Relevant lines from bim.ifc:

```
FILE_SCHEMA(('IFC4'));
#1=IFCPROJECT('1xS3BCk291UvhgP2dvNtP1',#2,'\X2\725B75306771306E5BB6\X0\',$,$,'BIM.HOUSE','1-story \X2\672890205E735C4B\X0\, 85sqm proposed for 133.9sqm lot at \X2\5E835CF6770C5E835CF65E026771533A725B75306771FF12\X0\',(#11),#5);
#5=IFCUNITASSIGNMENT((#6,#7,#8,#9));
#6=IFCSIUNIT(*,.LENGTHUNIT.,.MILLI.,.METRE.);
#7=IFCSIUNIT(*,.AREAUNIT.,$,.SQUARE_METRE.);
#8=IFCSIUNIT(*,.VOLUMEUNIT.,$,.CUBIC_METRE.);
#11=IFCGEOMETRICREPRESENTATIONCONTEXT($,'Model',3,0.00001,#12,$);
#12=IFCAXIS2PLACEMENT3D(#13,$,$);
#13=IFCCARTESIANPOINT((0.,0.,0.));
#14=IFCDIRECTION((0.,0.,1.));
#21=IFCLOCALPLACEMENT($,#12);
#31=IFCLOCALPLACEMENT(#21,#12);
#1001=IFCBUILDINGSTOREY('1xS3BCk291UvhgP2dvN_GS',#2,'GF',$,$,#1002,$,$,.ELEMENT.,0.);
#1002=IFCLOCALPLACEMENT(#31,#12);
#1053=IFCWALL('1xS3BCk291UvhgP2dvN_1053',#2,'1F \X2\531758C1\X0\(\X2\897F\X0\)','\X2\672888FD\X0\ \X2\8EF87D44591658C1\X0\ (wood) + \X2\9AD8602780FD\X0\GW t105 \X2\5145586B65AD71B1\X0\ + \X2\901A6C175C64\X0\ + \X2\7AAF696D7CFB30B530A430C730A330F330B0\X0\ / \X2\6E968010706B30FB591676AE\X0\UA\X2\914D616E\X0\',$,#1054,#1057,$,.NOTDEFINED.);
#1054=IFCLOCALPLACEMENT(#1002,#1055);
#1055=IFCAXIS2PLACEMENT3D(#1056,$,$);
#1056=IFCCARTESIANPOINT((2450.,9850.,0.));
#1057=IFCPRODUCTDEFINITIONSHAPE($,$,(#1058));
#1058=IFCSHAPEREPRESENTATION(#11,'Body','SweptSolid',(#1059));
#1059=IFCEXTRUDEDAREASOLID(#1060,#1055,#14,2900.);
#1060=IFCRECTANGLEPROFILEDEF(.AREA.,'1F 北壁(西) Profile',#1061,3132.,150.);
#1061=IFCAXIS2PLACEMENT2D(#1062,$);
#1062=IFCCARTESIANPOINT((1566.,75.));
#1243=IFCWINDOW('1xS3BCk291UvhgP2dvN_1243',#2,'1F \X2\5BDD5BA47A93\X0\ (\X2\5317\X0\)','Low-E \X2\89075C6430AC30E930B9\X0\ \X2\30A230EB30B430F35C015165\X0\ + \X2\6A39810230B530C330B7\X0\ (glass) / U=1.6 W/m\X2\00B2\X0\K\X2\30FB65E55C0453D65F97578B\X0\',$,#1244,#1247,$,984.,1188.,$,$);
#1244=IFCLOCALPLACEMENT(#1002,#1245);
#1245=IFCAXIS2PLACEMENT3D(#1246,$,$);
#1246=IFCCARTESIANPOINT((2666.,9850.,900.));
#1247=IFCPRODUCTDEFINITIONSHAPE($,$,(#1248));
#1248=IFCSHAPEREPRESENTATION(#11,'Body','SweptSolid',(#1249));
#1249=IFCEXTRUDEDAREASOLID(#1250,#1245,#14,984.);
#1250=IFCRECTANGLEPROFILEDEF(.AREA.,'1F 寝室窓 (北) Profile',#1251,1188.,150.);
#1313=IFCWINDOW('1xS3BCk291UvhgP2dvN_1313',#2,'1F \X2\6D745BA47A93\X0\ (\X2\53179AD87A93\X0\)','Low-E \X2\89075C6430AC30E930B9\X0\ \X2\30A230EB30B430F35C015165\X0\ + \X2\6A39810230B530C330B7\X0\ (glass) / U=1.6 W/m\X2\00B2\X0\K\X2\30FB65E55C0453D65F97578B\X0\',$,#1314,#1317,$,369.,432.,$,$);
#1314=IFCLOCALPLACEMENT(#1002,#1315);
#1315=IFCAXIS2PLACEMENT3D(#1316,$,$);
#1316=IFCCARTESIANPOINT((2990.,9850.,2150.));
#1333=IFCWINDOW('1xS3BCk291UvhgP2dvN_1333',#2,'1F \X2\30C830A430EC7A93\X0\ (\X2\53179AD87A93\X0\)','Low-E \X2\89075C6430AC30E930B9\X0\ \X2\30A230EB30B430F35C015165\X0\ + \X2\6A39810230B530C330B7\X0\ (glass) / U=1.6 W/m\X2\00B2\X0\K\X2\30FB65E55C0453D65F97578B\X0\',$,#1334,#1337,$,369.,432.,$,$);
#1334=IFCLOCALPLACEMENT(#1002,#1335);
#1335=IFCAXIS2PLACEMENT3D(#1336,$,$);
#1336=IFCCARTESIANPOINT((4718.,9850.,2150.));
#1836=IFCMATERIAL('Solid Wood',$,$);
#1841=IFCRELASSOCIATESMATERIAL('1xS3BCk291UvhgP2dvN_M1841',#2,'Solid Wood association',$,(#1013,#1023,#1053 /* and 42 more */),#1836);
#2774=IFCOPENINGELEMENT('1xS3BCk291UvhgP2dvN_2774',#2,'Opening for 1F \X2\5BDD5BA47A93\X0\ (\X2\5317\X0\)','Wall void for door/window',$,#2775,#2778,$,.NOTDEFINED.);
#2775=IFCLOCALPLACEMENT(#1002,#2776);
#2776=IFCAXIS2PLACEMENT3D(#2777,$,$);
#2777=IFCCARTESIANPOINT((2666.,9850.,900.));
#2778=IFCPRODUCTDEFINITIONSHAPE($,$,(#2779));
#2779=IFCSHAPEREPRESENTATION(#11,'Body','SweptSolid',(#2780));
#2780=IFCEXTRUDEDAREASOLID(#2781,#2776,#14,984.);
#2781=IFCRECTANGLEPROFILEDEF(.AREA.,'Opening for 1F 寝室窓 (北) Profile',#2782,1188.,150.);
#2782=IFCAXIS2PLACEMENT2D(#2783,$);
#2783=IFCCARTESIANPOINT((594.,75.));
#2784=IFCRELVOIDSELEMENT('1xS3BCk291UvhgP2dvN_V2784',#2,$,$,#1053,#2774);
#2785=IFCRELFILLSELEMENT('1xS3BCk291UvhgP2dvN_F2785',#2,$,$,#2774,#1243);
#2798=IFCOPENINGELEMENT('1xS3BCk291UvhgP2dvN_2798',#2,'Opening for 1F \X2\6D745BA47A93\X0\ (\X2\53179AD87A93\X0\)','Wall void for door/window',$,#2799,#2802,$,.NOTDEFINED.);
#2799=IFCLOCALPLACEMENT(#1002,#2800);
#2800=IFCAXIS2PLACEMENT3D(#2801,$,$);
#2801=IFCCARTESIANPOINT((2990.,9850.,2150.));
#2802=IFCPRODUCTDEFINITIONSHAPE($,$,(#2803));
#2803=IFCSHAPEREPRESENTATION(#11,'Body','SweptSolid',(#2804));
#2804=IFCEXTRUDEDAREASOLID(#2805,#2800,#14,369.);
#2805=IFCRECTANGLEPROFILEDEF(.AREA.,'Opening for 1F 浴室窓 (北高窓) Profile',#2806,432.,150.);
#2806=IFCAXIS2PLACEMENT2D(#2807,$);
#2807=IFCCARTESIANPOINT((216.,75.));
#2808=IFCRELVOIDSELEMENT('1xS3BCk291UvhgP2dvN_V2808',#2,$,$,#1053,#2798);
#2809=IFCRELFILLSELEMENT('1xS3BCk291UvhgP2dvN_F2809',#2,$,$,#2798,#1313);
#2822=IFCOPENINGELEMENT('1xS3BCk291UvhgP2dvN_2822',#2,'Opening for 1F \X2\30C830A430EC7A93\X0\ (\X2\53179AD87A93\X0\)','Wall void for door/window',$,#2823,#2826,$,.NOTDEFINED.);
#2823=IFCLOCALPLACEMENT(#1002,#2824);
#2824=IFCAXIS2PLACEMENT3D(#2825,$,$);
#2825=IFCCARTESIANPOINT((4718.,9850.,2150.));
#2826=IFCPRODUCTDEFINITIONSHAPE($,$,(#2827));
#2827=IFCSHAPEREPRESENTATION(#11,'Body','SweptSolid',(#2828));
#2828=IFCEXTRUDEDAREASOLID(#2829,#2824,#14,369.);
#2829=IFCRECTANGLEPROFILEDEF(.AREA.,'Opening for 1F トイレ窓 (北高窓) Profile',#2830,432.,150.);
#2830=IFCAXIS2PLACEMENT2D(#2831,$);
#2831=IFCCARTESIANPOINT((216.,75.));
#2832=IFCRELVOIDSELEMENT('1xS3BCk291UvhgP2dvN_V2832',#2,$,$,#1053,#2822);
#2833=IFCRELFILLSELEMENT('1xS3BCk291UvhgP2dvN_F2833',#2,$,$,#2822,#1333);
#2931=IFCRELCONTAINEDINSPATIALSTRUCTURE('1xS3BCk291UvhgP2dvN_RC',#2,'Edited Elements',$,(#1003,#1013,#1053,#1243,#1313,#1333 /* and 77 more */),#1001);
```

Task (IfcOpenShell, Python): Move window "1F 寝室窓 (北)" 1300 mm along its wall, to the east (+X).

```python
import ifcopenshell
import ifcopenshell.api.geometry
import ifcopenshell.util.placement

model = ifcopenshell.open("bim.ifc")

window = model.by_guid("1xS3BCk291UvhgP2dvN_1243")
opening = window.FillsVoids[0].RelatingOpeningElement
wall = opening.VoidsElements[0].RelatingBuildingElement

wall_matrix = ifcopenshell.util.placement.get_local_placement(wall.ObjectPlacement)
shift = wall_matrix[:3, 0] * 1300.0
before = ifcopenshell.util.placement.get_local_placement(window.ObjectPlacement)[:3, 3].copy()

# The window is not placed relative to its opening, so move both.
for product in (opening, window):
    matrix = ifcopenshell.util.placement.get_local_placement(product.ObjectPlacement)
    matrix[:3, 3] += shift
    ifcopenshell.api.geometry.edit_object_placement(model, product=product, matrix=matrix, is_si=False)

after = ifcopenshell.util.placement.get_local_placement(window.ObjectPlacement)[:3, 3]
print("window moved by", (after - before).round(3) + 0.0)

model.write("bim_updated.ifc")
```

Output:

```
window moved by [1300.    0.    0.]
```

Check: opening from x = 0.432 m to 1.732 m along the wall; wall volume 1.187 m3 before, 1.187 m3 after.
